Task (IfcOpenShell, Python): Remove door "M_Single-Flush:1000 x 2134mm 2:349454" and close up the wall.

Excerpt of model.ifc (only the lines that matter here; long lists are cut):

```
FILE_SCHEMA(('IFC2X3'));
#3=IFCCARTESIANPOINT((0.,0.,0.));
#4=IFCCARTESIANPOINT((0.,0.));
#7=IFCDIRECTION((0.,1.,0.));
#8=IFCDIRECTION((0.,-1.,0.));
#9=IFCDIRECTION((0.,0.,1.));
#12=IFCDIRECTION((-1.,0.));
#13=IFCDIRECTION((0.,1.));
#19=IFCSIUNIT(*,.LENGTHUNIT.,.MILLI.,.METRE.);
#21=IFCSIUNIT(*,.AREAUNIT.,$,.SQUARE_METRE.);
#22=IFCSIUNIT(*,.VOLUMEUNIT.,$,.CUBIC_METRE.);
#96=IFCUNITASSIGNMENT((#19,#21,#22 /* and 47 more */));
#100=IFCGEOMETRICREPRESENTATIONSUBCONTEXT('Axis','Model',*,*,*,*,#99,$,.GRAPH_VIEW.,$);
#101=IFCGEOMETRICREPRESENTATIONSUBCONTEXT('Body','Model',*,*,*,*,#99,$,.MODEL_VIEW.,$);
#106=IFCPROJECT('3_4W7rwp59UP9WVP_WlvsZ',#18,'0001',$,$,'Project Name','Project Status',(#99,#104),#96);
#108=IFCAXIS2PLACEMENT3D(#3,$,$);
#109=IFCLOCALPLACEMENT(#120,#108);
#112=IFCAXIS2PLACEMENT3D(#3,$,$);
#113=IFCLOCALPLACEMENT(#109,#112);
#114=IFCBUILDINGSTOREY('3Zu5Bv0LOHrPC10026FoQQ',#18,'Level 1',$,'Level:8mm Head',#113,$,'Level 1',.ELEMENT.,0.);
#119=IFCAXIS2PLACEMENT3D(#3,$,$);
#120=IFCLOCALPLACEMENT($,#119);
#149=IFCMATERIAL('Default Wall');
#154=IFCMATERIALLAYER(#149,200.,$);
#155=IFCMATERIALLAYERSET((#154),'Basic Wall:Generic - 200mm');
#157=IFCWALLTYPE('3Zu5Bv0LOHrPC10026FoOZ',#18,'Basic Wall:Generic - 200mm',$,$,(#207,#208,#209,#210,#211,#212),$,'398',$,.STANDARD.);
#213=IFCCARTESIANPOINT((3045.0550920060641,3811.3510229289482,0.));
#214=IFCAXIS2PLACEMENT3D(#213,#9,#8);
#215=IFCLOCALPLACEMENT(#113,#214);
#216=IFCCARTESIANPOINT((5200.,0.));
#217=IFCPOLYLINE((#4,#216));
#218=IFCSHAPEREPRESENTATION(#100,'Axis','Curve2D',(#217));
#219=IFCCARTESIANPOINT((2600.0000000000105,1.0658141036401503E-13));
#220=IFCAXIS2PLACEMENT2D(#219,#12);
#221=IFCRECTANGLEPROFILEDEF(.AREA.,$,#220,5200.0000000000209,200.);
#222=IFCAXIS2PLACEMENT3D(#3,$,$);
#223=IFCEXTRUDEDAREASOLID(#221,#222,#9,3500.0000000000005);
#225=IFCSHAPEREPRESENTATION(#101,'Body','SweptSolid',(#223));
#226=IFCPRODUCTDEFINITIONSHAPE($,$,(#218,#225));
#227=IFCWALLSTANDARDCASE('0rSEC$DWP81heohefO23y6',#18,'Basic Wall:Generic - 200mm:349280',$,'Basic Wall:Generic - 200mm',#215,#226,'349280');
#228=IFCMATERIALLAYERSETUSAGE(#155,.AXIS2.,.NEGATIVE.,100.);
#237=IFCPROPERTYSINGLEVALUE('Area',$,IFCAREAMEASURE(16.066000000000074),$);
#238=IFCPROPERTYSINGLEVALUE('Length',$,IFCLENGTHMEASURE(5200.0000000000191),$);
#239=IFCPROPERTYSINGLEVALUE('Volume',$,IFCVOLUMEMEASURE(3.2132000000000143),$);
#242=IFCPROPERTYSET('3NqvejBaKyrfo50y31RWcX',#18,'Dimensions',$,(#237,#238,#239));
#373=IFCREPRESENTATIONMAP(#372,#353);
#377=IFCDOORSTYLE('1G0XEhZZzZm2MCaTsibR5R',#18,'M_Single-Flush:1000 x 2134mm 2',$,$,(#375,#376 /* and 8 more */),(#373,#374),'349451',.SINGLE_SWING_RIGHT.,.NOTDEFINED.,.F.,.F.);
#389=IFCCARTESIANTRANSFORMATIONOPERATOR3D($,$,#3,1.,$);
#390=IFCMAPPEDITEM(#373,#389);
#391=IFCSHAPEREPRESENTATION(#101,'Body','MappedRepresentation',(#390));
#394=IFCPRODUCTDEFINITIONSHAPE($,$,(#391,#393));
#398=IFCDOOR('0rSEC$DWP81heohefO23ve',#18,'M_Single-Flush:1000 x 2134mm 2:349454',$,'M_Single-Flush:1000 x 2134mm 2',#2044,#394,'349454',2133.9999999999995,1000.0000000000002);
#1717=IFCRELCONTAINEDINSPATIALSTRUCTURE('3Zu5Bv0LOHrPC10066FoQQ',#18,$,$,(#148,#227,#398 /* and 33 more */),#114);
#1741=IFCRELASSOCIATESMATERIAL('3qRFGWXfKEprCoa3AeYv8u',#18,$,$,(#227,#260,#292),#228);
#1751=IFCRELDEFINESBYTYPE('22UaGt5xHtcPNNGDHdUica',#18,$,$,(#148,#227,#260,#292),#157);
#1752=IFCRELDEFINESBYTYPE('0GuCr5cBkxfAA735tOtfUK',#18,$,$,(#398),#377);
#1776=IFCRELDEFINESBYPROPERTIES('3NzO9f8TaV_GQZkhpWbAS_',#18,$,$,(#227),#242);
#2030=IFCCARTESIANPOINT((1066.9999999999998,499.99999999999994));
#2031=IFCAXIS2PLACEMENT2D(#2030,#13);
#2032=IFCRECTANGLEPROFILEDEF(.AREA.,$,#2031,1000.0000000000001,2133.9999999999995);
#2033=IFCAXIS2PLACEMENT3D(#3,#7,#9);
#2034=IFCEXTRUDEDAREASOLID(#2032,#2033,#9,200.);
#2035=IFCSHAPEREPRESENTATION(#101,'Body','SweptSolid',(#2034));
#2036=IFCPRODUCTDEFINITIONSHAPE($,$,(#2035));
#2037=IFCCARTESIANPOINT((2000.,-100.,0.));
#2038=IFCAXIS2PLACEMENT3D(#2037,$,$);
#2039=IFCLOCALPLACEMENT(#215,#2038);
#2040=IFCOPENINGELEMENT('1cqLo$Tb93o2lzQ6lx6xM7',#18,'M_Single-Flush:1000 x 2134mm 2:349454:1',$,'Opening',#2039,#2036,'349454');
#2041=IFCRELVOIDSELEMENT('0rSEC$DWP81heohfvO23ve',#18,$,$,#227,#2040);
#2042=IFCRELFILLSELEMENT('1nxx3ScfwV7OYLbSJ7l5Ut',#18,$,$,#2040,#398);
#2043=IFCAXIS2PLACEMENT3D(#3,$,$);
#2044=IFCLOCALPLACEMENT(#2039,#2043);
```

```python
import ifcopenshell
import ifcopenshell.api.feature
import ifcopenshell.api.pset
import ifcopenshell.api.root
import ifcopenshell.geom
import ifcopenshell.util.element
import ifcopenshell.util.shape
import ifcopenshell.util.unit

model = ifcopenshell.open("model.ifc")
area_scale = ifcopenshell.util.unit.calculate_unit_scale(model, "AREAUNIT")
volume_scale = ifcopenshell.util.unit.calculate_unit_scale(model, "VOLUMEUNIT")
settings = ifcopenshell.geom.settings()


def volume(element):
    """Net volume in cubic metres, openings subtracted."""
    shape = ifcopenshell.geom.create_shape(settings, element)
    return ifcopenshell.util.shape.get_volume(shape.geometry)


door = model.by_guid("0rSEC$DWP81heohefO23ve")
opening = door.FillsVoids[0].RelatingOpeningElement
wall = opening.VoidsElements[0].RelatingBuildingElement
before = volume(wall)

ifcopenshell.api.root.remove_product(model, product=door)
ifcopenshell.api.feature.remove_feature(model, feature=opening)

after = volume(wall)
thickness = 0.2  # wall thickness in metres

# Update the wall's stored quantities.
pset = model.by_id(ifcopenshell.util.element.get_pset(wall, "Dimensions", should_inherit=False)["id"])
ifcopenshell.api.pset.edit_pset(model, pset=pset, properties={
    "Area": model.create_entity("IfcAreaMeasure", after / thickness / area_scale),
    "Volume": model.create_entity("IfcVolumeMeasure", after / volume_scale),
})

print(f"wall volume {before:.3f} -> {after:.3f} m3")

model.write("model_edited.ifc")
```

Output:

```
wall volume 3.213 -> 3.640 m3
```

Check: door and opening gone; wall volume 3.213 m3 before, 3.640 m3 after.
